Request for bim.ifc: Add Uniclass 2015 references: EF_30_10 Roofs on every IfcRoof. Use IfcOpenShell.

First a look at what the model holds.

```python
import ifcopenshell

model = ifcopenshell.open("bim.ifc")
print(model.schema)
print("classifications:", [c.Name for c in model.by_type("IfcClassification")])
for ifc_class in ("IfcDoor", "IfcRoof", "IfcStair", "IfcWall", "IfcWindow"):
    print(ifc_class, len(model.by_type(ifc_class)))
```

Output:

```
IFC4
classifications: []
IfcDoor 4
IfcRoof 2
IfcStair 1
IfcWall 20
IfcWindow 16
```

```python
import ifcopenshell
import ifcopenshell.api.classification

model = ifcopenshell.open("bim.ifc")

system = ifcopenshell.api.classification.add_classification(model, classification="Uniclass 2015")

codes = {
    "IfcRoof": ("EF_30_10", "Roofs"),
}
for ifc_class, (code, name) in codes.items():
    products = model.by_type(ifc_class)
    ifcopenshell.api.classification.add_reference(
        model, products=products, classification=system, identification=code, name=name
    )
    print(code, len(products))

model.write("bim_v2.ifc")
```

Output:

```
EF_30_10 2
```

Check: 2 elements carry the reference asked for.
